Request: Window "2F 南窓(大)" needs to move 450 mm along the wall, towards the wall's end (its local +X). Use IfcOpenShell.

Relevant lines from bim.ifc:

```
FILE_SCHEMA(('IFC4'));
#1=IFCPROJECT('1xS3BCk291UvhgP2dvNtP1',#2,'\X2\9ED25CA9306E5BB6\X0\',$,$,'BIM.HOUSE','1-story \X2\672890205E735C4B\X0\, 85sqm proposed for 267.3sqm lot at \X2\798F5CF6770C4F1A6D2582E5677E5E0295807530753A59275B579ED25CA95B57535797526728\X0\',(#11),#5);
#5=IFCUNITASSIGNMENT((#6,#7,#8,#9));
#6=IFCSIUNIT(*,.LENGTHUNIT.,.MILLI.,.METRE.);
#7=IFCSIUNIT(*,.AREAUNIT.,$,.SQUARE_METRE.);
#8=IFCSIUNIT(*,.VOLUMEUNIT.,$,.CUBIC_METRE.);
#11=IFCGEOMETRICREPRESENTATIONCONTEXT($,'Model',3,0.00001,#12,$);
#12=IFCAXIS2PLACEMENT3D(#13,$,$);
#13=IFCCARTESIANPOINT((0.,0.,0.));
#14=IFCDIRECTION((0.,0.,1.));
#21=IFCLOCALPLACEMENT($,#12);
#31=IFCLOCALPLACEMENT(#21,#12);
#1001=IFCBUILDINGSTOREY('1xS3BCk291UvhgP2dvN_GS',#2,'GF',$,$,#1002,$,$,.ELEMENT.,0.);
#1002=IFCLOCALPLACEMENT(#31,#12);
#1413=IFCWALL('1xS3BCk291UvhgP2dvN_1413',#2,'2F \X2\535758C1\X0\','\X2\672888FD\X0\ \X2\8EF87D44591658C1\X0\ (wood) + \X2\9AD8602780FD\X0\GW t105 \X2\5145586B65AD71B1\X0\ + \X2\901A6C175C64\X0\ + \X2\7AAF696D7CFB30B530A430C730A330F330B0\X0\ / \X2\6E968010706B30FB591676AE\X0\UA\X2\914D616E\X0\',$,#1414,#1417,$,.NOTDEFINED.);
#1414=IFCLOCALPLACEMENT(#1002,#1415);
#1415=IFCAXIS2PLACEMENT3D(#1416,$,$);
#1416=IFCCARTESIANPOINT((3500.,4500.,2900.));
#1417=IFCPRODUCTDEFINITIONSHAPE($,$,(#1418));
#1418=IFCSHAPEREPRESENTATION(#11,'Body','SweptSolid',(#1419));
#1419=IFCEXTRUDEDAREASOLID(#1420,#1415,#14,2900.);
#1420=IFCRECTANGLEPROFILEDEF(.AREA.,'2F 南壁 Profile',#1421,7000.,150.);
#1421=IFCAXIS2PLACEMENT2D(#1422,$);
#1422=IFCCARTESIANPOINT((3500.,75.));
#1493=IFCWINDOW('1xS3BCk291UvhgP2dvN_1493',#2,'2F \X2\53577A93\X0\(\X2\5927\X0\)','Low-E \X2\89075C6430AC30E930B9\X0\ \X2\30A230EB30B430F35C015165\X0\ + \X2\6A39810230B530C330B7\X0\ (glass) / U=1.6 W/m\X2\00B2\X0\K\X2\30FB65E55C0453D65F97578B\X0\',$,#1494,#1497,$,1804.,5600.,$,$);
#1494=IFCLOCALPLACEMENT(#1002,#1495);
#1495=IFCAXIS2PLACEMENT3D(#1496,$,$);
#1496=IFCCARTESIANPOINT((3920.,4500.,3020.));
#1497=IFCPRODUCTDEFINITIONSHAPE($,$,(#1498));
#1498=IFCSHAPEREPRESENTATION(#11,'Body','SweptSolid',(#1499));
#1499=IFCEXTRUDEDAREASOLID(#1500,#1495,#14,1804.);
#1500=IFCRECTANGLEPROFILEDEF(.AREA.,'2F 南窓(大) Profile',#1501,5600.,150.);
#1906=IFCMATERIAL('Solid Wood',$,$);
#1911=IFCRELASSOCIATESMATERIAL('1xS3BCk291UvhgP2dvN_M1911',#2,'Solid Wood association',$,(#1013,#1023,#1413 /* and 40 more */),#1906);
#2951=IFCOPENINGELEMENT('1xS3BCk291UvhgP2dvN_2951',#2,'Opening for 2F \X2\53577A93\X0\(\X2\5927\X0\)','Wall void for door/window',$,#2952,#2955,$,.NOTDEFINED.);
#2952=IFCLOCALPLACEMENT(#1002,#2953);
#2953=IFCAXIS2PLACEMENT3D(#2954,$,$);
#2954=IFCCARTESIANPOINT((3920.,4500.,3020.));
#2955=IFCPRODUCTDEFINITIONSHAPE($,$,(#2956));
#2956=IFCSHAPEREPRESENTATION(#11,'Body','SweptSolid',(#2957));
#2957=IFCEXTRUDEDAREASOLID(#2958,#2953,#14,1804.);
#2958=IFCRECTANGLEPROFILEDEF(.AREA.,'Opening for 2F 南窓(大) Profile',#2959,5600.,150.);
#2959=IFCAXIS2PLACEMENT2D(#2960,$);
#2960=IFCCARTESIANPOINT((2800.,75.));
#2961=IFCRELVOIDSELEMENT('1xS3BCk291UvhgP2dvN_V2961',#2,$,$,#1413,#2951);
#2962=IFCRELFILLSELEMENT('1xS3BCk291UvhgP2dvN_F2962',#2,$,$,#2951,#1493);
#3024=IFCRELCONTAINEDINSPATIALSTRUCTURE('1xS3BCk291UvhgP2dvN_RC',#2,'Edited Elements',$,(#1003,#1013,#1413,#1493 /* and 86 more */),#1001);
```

```python
import ifcopenshell
import ifcopenshell.api.geometry
import ifcopenshell.util.placement

model = ifcopenshell.open("bim.ifc")

window = model.by_id(1493)
opening = window.FillsVoids[0].RelatingOpeningElement
wall = opening.VoidsElements[0].RelatingBuildingElement

wall_matrix = ifcopenshell.util.placement.get_local_placement(wall.ObjectPlacement)
shift = wall_matrix[:3, 0] * 450.0
before = ifcopenshell.util.placement.get_local_placement(window.ObjectPlacement)[:3, 3].copy()

# The window is not placed relative to its opening, so move both.
for product in (opening, window):
    matrix = ifcopenshell.util.placement.get_local_placement(product.ObjectPlacement)
    matrix[:3, 3] += shift
    ifcopenshell.api.geometry.edit_object_placement(model, product=product, matrix=matrix, is_si=False)

after = ifcopenshell.util.placement.get_local_placement(window.ObjectPlacement)[:3, 3]
print("window moved by", (after - before).round(3) + 0.0)

model.write("bim_v2.ifc")
```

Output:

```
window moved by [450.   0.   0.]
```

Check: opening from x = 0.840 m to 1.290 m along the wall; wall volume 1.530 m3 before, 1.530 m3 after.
